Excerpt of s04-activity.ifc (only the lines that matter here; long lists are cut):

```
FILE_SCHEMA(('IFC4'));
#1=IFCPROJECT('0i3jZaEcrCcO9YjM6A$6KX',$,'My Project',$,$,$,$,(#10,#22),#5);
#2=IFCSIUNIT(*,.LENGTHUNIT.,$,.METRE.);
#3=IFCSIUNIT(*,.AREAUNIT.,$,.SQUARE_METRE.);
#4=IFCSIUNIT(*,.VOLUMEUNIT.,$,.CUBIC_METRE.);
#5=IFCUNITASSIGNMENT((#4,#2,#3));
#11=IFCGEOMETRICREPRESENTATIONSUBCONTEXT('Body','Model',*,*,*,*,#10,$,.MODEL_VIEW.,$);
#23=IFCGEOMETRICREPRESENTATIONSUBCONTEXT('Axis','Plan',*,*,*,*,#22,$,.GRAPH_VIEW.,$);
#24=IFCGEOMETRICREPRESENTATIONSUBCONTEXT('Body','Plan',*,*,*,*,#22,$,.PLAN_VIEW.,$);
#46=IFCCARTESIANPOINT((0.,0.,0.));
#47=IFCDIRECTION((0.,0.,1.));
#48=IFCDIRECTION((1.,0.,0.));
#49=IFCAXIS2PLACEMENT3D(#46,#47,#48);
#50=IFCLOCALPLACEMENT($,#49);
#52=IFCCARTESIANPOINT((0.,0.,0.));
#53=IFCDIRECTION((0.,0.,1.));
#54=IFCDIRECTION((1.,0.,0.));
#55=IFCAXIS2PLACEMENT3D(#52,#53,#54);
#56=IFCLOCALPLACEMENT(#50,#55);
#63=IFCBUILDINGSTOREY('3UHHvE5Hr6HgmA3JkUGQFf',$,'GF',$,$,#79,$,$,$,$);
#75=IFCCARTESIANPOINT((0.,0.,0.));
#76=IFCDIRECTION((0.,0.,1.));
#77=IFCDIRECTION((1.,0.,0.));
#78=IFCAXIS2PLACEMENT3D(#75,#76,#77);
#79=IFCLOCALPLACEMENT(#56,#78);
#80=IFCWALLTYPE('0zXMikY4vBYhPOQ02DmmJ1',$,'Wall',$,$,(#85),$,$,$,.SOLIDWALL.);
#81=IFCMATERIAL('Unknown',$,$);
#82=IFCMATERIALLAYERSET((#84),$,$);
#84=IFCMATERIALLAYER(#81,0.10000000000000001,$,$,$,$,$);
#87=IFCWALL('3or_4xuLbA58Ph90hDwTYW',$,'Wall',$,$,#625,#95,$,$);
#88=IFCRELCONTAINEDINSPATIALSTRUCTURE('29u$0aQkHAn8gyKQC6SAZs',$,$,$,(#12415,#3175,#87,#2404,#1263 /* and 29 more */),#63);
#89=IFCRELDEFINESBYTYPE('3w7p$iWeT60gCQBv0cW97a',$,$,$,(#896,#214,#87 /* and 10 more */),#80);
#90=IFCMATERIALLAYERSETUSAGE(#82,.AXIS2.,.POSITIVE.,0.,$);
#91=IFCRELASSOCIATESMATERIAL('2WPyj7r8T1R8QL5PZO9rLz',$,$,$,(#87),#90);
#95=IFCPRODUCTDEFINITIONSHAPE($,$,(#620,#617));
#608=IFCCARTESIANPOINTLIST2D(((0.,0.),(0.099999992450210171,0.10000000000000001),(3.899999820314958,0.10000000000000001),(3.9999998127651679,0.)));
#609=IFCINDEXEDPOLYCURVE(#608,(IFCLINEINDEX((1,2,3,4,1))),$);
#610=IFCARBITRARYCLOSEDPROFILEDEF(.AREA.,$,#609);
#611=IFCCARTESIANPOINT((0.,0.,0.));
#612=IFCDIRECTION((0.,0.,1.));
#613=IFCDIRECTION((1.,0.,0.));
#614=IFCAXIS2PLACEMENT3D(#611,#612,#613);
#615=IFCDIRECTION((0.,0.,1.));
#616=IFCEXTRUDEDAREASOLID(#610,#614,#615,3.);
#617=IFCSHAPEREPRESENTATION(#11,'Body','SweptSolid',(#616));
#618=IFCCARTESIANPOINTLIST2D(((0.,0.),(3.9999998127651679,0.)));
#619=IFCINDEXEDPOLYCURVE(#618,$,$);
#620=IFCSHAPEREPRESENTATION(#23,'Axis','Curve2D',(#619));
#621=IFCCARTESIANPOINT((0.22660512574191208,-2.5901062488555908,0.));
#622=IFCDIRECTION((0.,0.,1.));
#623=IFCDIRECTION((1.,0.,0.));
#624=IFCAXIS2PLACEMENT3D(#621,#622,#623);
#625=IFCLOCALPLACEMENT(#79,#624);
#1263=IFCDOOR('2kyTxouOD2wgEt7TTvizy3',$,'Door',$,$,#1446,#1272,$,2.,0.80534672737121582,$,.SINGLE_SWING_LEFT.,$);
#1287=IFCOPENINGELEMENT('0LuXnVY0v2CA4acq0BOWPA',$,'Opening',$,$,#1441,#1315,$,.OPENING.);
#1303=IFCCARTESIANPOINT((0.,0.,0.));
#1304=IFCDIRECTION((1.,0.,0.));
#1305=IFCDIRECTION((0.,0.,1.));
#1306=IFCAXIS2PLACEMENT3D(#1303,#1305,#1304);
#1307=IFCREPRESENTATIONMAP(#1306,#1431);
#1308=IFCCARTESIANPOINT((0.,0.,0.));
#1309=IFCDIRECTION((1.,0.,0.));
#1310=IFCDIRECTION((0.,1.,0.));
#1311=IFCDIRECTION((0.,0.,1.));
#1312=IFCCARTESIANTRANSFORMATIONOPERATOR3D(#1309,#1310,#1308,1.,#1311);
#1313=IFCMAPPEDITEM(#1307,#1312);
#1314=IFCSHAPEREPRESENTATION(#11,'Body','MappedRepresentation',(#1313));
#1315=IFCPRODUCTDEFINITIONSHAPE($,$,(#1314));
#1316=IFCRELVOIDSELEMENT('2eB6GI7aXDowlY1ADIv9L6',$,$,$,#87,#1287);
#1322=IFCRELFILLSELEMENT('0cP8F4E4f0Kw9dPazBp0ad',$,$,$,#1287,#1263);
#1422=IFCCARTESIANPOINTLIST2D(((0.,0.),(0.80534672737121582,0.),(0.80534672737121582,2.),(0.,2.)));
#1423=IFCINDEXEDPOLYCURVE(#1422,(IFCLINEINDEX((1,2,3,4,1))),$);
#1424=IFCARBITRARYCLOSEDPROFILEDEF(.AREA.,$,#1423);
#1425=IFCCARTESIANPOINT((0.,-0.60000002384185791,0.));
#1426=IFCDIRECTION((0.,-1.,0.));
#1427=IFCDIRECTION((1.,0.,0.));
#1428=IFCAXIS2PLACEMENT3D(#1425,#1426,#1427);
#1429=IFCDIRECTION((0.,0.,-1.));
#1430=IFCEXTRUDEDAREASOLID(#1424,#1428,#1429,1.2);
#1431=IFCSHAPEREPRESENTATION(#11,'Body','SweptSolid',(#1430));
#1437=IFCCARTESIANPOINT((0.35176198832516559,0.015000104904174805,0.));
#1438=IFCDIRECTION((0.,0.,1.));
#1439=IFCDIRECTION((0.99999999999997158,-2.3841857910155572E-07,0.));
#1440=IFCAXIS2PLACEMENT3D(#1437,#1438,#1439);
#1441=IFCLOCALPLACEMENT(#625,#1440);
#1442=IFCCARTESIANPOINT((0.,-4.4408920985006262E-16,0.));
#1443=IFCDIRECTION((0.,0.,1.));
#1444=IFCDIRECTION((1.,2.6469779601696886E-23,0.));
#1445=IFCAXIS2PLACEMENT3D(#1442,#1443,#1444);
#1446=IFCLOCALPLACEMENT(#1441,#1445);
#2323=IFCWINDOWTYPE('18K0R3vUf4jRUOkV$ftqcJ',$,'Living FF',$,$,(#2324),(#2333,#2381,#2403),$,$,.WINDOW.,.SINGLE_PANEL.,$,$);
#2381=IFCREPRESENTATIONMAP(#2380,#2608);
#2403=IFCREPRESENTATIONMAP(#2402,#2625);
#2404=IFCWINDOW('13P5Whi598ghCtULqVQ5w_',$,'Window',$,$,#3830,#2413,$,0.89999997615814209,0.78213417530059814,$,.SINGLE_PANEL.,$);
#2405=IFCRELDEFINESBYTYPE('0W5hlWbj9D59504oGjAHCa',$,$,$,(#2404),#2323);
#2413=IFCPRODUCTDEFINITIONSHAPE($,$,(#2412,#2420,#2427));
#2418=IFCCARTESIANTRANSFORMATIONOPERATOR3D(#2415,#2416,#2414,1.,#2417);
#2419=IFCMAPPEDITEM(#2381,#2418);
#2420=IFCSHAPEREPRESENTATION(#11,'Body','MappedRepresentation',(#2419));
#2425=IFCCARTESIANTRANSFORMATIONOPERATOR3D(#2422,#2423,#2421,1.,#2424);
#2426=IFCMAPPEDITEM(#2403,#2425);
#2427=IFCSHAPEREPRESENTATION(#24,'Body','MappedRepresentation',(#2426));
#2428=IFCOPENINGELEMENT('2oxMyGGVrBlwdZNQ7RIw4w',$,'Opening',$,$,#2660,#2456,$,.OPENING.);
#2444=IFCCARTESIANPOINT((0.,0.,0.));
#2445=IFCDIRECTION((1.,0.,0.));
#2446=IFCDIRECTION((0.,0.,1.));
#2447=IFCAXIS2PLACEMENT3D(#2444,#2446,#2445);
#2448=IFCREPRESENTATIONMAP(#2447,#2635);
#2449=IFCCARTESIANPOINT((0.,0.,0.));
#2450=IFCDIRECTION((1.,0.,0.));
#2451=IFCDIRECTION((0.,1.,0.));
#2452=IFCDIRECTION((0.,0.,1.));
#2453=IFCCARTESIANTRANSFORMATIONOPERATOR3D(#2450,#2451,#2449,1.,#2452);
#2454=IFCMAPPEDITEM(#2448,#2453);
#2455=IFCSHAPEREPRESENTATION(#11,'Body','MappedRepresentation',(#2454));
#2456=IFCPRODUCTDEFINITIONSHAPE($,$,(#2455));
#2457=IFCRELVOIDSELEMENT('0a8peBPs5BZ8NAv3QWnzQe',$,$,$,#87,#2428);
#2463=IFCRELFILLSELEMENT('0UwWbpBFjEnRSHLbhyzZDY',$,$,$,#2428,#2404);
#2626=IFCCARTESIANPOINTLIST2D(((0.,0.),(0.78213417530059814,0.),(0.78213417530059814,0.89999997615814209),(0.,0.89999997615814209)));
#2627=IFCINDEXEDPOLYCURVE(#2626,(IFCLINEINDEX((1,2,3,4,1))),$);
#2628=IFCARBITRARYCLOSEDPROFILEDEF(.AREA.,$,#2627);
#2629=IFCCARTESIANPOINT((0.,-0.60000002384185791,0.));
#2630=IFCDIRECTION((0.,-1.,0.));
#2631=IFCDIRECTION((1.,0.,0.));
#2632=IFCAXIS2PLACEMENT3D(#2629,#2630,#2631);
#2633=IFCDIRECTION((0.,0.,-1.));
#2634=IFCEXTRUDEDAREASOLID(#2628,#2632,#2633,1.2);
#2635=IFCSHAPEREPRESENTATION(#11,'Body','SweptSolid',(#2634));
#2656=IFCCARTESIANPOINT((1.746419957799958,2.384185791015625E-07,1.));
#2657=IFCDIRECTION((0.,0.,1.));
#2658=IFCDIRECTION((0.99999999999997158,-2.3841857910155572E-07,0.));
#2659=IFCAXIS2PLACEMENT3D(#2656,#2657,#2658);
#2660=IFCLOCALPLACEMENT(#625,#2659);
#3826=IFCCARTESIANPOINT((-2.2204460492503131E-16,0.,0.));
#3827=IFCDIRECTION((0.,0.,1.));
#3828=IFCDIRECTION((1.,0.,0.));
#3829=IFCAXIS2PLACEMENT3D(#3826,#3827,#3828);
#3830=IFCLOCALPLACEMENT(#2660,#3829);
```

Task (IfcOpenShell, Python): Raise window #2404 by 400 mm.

```python
import numpy as np
import ifcopenshell
import ifcopenshell.api.geometry
import ifcopenshell.util.placement
import ifcopenshell.util.unit

model = ifcopenshell.open("s04-activity.ifc")
unit_scale = ifcopenshell.util.unit.calculate_unit_scale(model)

window = model.by_guid("13P5Whi598ghCtULqVQ5w_")
opening = window.FillsVoids[0].RelatingOpeningElement
dz = 0.4 / unit_scale

shift = np.array([0.0, 0.0, dz])
# The window is placed relative to its opening, so it follows when the opening moves.
matrix = ifcopenshell.util.placement.get_local_placement(opening.ObjectPlacement)
matrix[:3, 3] += shift
ifcopenshell.api.geometry.edit_object_placement(
    model, product=opening, matrix=matrix, is_si=False, should_transform_children=True
)

print(f"moved by {dz * unit_scale:+.3f} m")

model.write("s04-activity_updated.ifc")
```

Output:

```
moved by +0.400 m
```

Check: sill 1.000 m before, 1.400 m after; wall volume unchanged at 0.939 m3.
